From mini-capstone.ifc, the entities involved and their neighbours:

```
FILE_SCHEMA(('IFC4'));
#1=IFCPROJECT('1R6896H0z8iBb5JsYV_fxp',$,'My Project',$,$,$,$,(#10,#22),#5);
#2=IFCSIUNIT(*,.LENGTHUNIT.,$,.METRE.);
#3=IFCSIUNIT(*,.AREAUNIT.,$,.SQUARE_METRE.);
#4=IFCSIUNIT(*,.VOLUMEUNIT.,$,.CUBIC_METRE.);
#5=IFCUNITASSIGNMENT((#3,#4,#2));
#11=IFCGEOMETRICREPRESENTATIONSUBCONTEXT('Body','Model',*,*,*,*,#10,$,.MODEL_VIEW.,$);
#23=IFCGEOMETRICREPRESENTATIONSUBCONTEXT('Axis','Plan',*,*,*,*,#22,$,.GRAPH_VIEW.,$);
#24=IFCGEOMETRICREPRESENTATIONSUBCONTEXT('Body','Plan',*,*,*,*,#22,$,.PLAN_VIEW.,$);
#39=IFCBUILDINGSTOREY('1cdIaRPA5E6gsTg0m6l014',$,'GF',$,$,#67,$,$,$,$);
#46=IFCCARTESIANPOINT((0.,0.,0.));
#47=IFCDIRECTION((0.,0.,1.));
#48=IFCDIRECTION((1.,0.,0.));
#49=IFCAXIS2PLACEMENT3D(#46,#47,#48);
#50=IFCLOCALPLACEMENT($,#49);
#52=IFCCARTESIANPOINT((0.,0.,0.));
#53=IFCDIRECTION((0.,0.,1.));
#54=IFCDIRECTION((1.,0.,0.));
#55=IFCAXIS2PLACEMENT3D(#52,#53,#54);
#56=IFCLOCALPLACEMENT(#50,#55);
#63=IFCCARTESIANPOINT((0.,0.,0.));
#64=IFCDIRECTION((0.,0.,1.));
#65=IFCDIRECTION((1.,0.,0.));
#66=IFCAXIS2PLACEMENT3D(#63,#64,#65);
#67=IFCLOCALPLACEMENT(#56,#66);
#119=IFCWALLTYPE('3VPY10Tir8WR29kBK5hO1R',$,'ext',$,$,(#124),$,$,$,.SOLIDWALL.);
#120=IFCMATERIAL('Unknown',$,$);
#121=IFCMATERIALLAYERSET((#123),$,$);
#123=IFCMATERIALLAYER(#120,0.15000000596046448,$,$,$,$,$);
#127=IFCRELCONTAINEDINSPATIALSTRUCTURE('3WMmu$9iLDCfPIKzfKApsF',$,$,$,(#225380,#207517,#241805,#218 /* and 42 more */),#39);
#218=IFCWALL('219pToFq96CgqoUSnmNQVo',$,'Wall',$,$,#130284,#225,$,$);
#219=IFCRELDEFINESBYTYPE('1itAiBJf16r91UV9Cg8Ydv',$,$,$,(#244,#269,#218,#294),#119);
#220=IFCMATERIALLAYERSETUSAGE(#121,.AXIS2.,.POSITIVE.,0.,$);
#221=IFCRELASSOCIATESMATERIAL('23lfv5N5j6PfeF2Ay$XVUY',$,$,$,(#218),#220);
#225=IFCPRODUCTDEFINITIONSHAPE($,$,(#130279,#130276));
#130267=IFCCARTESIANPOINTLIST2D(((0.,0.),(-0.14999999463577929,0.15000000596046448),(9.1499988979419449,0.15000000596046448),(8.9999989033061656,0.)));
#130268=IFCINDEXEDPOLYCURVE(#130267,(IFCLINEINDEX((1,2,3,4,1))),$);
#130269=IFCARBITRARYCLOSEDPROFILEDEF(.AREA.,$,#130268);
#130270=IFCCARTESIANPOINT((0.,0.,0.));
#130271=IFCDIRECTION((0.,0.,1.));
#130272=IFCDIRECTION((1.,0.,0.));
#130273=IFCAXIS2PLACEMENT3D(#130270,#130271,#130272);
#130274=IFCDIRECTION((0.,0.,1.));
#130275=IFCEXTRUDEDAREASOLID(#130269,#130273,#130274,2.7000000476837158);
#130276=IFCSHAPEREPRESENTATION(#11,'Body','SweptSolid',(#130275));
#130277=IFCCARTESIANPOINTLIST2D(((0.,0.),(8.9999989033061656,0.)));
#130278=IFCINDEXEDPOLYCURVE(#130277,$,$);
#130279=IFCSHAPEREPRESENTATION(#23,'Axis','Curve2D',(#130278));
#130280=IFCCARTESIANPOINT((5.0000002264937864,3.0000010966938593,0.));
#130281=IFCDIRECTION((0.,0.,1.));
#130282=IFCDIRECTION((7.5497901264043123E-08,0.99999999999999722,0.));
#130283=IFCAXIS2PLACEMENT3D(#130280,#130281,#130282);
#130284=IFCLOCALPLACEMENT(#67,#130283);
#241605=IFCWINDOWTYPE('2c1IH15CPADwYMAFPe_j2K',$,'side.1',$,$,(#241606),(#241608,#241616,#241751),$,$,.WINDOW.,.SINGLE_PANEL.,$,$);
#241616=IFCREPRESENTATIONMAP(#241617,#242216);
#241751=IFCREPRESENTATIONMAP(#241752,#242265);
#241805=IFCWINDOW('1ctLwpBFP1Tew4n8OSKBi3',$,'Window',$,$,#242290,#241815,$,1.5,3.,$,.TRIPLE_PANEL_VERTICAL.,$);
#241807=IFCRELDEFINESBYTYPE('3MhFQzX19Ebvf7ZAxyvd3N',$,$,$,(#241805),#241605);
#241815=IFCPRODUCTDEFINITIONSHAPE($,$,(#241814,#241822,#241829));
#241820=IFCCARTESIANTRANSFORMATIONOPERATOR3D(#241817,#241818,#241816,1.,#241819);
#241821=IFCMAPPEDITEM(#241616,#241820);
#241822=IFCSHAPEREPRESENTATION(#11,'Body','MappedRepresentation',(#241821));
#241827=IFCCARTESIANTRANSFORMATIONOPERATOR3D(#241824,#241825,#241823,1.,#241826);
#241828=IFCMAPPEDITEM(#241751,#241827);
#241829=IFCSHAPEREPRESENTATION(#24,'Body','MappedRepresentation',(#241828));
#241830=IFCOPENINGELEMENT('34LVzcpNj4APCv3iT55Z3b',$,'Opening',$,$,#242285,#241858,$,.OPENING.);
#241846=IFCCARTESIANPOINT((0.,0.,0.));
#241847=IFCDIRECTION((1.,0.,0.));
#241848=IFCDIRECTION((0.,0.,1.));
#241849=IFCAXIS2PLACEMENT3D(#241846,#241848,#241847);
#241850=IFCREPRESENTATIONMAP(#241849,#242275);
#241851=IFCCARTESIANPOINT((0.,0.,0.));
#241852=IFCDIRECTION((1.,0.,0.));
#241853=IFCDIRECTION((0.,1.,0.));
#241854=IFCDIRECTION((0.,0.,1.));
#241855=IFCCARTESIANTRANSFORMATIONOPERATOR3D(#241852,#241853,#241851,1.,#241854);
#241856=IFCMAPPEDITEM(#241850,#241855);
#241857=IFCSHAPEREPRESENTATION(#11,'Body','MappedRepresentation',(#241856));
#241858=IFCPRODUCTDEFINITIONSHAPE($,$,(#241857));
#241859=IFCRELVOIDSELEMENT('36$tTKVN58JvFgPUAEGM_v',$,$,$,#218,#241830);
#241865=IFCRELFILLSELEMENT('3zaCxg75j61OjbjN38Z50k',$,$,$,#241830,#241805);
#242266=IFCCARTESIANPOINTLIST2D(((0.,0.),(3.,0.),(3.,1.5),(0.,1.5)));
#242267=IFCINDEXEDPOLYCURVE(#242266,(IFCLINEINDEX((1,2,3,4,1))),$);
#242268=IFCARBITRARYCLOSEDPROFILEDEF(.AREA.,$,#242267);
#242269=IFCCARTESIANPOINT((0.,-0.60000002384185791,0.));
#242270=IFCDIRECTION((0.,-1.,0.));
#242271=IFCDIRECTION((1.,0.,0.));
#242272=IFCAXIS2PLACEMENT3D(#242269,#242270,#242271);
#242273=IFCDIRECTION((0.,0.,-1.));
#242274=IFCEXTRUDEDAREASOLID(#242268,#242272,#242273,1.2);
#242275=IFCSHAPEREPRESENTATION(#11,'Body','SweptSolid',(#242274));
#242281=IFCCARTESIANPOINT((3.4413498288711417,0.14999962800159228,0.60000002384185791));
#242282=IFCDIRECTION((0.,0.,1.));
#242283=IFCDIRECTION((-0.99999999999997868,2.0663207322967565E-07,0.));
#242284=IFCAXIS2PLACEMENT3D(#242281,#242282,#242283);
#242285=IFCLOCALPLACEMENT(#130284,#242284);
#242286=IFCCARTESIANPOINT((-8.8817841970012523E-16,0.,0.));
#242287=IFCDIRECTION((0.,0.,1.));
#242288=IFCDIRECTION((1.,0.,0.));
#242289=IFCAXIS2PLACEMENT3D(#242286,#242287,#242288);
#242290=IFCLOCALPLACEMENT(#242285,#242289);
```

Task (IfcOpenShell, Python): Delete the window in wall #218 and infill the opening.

```python
import ifcopenshell
import ifcopenshell.api.feature
import ifcopenshell.api.root
import ifcopenshell.geom
import ifcopenshell.util.shape

model = ifcopenshell.open("mini-capstone.ifc")
settings = ifcopenshell.geom.settings()


def volume(element):
    """Net volume in cubic metres, openings subtracted."""
    shape = ifcopenshell.geom.create_shape(settings, element)
    return ifcopenshell.util.shape.get_volume(shape.geometry)


window = model.by_guid("1ctLwpBFP1Tew4n8OSKBi3")
opening = window.FillsVoids[0].RelatingOpeningElement
wall = opening.VoidsElements[0].RelatingBuildingElement
before = volume(wall)

ifcopenshell.api.root.remove_product(model, product=window)
ifcopenshell.api.feature.remove_feature(model, feature=opening)

after = volume(wall)

print(f"wall volume {before:.3f} -> {after:.3f} m3")

model.write("mini-capstone_rev.ifc")
```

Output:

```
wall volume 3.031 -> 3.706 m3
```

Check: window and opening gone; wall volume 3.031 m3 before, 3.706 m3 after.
